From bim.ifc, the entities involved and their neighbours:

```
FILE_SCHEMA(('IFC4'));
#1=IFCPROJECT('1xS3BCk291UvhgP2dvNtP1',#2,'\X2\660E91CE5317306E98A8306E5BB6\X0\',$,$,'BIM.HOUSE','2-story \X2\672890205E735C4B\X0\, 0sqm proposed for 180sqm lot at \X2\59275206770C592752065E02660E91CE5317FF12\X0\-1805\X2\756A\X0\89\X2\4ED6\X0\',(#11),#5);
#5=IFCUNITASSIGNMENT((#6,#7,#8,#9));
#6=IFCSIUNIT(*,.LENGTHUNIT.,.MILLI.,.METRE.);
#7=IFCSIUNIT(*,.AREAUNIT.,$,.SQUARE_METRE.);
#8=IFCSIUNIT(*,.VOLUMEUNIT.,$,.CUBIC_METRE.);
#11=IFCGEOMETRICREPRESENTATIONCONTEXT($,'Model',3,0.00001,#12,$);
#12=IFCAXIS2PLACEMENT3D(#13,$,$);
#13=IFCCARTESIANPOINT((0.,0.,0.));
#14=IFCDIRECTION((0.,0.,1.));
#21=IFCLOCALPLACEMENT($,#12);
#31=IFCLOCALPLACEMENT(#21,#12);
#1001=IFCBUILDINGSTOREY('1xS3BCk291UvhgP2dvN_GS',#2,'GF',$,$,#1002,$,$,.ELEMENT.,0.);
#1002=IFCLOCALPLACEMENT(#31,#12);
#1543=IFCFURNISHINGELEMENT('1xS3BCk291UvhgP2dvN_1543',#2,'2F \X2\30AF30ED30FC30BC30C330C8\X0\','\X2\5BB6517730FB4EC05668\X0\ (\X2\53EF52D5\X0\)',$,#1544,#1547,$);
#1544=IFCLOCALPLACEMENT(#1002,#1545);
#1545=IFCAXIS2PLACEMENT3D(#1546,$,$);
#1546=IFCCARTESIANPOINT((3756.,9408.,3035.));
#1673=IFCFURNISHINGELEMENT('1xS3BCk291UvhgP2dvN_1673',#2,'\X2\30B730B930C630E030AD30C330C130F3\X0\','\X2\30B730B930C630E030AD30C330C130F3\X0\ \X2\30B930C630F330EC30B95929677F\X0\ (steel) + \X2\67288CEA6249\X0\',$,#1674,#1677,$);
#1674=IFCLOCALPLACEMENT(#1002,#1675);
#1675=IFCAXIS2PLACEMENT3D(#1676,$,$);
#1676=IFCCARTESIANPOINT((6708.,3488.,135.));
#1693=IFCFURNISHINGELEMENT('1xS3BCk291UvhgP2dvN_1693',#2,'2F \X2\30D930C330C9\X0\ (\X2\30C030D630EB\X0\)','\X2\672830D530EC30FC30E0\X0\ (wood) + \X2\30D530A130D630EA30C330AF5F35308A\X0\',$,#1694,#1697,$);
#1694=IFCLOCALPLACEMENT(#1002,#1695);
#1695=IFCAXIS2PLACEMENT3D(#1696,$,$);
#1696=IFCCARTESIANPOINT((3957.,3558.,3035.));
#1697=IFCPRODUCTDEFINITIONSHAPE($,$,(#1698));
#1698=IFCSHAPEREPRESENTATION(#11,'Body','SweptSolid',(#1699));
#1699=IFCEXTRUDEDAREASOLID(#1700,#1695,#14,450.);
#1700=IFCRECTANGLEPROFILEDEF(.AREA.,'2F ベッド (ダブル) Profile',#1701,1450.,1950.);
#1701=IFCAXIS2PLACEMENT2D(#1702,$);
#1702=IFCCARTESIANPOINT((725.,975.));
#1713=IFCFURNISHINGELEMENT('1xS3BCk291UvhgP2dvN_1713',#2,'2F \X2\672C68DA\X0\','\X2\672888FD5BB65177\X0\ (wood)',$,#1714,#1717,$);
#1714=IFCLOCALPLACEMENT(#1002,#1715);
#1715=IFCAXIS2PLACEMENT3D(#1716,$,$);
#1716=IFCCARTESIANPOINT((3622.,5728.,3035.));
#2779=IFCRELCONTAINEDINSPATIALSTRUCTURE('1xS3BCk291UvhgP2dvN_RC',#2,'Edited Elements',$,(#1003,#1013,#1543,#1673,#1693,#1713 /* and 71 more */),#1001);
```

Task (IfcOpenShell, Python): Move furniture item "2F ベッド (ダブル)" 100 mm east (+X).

```python
import ifcopenshell
import ifcopenshell.api.geometry
import ifcopenshell.util.placement

model = ifcopenshell.open("bim.ifc")

item = model.by_guid("1xS3BCk291UvhgP2dvN_1693")
matrix = ifcopenshell.util.placement.get_local_placement(item.ObjectPlacement)
matrix[0, 3] += 100.0
ifcopenshell.api.geometry.edit_object_placement(model, product=item, matrix=matrix, is_si=False)

print(ifcopenshell.util.placement.get_local_placement(item.ObjectPlacement).round(3) + 0.0)

model.write("bim_v2.ifc")
```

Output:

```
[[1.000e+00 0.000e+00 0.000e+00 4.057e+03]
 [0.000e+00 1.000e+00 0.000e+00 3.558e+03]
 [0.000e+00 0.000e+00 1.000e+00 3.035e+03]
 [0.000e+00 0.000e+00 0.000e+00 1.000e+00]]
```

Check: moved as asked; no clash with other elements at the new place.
